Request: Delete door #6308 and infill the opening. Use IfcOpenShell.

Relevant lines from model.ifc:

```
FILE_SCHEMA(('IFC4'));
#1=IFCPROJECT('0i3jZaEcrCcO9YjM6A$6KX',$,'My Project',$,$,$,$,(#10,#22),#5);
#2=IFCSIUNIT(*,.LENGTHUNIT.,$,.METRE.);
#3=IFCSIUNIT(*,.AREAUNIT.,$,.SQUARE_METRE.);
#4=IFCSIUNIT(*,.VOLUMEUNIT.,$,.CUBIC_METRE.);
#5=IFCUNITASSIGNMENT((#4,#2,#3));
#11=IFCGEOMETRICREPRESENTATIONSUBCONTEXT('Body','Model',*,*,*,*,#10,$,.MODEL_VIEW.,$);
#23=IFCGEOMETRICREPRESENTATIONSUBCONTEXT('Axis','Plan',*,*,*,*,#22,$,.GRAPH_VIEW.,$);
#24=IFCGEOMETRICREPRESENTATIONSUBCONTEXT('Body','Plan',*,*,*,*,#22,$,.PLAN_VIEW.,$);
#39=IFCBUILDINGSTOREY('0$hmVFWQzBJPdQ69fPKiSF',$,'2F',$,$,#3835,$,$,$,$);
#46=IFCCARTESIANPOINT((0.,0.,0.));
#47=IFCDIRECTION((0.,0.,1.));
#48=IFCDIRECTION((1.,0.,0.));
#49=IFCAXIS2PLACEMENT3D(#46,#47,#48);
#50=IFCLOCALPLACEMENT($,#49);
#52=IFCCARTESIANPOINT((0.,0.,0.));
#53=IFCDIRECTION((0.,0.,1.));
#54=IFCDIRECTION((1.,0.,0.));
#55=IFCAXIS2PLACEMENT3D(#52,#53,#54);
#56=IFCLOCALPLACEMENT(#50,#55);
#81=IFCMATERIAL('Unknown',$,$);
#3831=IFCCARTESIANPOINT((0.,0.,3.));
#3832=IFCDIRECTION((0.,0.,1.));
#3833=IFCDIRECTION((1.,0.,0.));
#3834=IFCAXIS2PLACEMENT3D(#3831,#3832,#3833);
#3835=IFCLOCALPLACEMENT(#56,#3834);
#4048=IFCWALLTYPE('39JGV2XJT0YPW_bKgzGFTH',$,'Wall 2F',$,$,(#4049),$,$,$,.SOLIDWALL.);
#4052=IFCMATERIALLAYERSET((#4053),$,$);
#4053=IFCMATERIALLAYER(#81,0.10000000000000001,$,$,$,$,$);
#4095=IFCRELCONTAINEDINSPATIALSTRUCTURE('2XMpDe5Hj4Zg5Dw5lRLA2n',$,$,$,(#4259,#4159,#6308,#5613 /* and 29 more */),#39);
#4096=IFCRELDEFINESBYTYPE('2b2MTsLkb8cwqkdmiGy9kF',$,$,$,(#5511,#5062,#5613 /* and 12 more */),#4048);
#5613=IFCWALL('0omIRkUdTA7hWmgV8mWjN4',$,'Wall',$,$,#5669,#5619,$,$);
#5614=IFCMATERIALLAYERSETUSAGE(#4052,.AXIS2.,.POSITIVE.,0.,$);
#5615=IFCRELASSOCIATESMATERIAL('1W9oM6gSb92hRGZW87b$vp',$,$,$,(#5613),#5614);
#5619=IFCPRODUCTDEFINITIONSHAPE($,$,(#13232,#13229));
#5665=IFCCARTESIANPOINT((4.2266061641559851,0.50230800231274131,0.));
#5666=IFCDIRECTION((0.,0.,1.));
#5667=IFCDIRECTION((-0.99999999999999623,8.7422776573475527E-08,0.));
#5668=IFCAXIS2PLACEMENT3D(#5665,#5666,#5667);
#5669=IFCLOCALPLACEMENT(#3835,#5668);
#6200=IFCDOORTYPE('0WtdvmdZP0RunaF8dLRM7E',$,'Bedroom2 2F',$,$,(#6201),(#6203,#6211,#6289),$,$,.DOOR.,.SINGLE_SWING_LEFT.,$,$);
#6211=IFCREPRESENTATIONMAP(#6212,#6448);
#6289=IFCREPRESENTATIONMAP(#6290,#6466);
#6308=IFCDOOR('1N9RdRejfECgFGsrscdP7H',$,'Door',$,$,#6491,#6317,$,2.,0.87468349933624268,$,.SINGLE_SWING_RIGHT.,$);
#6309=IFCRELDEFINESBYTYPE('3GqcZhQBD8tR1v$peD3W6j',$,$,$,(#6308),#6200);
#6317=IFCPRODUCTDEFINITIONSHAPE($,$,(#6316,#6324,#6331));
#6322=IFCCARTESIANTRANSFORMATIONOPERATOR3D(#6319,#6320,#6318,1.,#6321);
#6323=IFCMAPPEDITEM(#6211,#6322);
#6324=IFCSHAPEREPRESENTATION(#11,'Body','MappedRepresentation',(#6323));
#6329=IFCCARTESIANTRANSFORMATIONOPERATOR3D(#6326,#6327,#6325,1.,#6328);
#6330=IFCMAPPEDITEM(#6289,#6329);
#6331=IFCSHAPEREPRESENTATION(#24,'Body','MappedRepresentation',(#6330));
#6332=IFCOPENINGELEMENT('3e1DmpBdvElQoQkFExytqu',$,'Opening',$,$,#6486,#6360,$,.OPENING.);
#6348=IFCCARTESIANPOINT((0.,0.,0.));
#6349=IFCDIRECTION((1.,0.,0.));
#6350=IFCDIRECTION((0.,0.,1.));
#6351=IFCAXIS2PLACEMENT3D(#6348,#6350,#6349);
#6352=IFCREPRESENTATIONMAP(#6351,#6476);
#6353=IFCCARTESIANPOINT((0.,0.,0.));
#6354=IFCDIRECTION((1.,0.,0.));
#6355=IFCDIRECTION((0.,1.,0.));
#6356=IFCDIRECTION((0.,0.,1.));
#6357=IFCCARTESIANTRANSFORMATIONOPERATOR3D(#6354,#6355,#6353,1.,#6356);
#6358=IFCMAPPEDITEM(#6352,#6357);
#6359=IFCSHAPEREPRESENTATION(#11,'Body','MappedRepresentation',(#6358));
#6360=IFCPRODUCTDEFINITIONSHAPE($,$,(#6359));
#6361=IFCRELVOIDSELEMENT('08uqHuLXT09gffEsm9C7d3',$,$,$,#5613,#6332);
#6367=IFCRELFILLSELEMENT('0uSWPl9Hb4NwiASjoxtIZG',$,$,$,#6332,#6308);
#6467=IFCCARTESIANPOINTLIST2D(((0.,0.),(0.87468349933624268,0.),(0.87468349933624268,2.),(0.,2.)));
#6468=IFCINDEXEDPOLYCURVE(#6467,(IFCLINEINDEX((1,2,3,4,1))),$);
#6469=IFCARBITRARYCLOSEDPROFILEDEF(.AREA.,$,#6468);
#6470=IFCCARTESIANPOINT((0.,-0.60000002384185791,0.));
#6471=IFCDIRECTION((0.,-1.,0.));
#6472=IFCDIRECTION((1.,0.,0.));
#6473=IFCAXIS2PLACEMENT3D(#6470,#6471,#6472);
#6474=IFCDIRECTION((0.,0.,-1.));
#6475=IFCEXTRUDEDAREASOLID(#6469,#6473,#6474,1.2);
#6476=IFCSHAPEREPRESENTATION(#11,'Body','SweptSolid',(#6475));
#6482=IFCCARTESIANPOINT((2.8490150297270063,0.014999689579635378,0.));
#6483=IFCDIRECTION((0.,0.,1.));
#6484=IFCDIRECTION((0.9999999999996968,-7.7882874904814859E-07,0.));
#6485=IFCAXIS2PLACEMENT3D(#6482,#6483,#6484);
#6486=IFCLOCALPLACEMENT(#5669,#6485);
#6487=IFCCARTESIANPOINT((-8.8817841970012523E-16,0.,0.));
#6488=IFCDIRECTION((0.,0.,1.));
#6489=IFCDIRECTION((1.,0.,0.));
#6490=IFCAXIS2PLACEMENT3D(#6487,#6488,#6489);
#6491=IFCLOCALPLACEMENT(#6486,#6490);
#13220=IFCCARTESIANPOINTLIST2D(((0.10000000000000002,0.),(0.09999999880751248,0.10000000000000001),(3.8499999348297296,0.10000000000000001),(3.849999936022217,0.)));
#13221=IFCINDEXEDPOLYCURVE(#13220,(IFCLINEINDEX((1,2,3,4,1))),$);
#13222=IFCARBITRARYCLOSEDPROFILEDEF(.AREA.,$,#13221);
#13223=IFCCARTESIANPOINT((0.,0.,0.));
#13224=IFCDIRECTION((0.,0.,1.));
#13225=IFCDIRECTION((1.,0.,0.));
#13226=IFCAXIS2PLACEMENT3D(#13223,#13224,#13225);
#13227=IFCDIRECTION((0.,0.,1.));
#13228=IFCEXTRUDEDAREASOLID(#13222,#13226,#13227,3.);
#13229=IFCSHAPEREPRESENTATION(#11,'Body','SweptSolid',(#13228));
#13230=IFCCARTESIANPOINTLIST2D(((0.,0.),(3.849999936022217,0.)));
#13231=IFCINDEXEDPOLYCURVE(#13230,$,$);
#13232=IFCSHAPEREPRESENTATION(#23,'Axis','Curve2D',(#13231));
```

```python
import ifcopenshell
import ifcopenshell.api.feature
import ifcopenshell.api.root
import ifcopenshell.geom
import ifcopenshell.util.shape

model = ifcopenshell.open("model.ifc")
settings = ifcopenshell.geom.settings()


def volume(element):
    """Net volume in cubic metres, openings subtracted."""
    shape = ifcopenshell.geom.create_shape(settings, element)
    return ifcopenshell.util.shape.get_volume(shape.geometry)


door = model.by_guid("1N9RdRejfECgFGsrscdP7H")
opening = door.FillsVoids[0].RelatingOpeningElement
wall = opening.VoidsElements[0].RelatingBuildingElement
before = volume(wall)

ifcopenshell.api.root.remove_product(model, product=door)
ifcopenshell.api.feature.remove_feature(model, feature=opening)

after = volume(wall)

print(f"wall volume {before:.3f} -> {after:.3f} m3")

model.write("model_v2.ifc")
```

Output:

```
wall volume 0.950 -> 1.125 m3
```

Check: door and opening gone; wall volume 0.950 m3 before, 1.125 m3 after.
